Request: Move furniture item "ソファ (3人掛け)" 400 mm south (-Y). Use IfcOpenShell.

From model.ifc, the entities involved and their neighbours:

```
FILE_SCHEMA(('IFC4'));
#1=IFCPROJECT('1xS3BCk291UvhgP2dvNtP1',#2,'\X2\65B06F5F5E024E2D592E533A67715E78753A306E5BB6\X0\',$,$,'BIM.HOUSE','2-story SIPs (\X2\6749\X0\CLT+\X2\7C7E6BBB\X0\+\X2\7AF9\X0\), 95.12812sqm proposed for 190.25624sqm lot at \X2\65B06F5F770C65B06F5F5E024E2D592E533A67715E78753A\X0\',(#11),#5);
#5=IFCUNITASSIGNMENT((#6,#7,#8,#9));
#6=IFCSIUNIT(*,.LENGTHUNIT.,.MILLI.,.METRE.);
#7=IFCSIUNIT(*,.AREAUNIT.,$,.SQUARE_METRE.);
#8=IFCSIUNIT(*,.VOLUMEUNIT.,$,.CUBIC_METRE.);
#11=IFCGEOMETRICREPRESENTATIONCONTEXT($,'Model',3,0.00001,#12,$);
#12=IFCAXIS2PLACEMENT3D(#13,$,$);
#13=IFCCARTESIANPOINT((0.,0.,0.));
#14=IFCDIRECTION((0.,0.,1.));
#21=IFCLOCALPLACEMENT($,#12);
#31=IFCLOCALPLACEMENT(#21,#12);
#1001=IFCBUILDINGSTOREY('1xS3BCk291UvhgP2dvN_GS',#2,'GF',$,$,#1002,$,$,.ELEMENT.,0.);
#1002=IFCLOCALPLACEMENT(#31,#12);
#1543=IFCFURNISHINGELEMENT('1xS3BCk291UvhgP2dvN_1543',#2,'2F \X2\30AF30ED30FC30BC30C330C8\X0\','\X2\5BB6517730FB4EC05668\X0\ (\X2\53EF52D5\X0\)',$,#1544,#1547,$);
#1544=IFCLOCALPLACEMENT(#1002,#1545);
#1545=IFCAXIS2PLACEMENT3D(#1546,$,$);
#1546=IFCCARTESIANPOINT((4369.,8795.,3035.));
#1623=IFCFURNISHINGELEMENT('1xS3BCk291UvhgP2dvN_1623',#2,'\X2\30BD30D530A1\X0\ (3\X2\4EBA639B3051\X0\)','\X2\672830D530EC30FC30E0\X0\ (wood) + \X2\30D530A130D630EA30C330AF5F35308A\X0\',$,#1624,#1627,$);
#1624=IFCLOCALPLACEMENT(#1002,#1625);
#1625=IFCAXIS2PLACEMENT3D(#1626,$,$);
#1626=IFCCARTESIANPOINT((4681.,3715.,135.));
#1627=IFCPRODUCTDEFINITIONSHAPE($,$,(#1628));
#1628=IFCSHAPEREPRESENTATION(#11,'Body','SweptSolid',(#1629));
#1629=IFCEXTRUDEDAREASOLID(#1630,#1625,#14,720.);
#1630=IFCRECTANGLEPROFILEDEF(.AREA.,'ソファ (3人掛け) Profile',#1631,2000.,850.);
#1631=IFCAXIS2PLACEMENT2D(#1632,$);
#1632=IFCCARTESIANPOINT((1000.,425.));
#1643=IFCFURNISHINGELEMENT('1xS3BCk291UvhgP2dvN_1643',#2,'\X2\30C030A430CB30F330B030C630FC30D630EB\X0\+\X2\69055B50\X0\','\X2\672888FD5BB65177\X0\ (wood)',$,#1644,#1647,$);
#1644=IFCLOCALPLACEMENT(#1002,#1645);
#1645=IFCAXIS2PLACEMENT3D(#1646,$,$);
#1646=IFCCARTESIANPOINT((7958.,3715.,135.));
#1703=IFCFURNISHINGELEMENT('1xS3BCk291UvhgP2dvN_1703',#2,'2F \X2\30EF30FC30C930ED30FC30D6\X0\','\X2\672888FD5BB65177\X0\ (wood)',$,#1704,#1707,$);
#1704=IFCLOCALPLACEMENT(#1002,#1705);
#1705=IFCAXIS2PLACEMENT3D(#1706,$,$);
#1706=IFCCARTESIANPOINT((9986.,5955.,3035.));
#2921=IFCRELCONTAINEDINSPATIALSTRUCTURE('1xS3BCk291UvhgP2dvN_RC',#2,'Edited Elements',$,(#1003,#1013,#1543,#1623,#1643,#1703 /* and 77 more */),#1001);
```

```python
import ifcopenshell
import ifcopenshell.api.geometry
import ifcopenshell.util.placement
import ifcopenshell.util.unit

model = ifcopenshell.open("model.ifc")
unit_scale = ifcopenshell.util.unit.calculate_unit_scale(model)

item = model.by_guid("1xS3BCk291UvhgP2dvN_1623")
matrix = ifcopenshell.util.placement.get_local_placement(item.ObjectPlacement)
matrix[1, 3] -= 0.4 / unit_scale
ifcopenshell.api.geometry.edit_object_placement(model, product=item, matrix=matrix, is_si=False)

print(ifcopenshell.util.placement.get_local_placement(item.ObjectPlacement).round(3) + 0.0)

model.write("model_edited.ifc")
```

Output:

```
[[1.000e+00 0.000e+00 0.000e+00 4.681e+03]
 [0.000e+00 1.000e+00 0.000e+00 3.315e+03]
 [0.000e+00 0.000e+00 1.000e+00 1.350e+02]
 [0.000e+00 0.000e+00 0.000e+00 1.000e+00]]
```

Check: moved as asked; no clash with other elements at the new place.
